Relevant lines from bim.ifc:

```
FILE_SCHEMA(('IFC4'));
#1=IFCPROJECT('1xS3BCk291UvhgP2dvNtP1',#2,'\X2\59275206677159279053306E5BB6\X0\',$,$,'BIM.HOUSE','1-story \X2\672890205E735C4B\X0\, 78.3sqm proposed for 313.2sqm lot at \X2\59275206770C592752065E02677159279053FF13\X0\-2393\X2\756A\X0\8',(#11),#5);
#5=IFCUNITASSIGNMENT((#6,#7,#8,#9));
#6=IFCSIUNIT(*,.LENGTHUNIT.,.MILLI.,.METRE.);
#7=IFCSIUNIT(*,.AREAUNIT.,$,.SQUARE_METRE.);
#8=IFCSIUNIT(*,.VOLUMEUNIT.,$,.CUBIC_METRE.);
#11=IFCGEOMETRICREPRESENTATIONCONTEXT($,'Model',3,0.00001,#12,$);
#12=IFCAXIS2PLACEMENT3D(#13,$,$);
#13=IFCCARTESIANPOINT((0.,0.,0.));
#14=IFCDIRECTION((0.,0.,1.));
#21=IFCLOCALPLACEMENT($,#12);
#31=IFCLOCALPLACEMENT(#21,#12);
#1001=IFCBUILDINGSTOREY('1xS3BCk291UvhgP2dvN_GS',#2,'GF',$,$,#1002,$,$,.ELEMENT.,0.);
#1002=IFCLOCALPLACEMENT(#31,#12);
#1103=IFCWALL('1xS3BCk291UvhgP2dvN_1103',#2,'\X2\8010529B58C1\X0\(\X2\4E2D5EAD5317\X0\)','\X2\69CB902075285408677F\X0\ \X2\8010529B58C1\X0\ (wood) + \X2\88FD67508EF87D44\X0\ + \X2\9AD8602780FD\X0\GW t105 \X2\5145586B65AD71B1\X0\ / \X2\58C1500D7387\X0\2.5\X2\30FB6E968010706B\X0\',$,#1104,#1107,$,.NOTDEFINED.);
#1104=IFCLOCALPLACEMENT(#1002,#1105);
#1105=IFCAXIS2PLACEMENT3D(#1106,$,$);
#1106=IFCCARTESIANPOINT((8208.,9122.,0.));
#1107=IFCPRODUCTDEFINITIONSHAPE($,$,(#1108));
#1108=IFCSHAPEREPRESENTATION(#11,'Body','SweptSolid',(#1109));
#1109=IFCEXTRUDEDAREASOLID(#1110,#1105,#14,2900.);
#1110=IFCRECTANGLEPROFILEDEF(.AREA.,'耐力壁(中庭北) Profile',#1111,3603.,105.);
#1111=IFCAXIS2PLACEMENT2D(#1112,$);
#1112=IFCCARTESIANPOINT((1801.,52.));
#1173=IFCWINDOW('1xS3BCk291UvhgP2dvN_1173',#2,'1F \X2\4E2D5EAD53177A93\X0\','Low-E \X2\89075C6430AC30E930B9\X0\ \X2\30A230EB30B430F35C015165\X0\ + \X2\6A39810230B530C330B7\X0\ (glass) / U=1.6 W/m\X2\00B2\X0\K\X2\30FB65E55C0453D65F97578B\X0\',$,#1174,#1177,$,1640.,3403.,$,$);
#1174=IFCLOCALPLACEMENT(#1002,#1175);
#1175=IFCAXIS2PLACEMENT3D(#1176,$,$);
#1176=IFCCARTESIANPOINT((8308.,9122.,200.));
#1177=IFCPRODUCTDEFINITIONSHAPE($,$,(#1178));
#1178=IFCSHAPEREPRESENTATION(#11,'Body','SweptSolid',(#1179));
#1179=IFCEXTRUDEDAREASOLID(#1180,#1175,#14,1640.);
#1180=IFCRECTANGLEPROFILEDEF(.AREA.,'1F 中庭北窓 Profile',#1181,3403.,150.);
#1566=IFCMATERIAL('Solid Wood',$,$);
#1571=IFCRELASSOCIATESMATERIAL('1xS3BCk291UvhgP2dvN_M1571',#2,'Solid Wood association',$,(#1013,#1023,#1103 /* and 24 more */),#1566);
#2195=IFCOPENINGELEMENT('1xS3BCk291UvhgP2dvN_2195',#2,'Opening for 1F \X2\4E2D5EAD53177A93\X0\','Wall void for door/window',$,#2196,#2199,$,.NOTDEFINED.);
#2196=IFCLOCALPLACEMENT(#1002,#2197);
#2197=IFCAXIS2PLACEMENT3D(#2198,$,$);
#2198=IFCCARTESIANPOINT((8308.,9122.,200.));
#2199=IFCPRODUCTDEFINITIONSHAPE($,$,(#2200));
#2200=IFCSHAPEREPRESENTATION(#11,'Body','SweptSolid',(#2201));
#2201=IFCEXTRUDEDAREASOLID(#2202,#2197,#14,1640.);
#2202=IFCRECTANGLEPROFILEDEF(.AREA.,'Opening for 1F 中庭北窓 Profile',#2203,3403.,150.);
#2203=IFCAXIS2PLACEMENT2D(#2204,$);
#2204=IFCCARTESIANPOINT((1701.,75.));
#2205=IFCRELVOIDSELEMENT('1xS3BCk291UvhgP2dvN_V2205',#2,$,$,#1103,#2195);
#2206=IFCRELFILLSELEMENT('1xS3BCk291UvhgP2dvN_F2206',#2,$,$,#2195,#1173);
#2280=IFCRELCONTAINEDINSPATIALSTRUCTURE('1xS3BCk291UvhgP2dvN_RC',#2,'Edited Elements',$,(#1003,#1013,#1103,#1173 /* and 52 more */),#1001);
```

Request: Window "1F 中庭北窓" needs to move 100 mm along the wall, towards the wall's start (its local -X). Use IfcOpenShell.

```python
import ifcopenshell
import ifcopenshell.api.geometry
import ifcopenshell.util.placement
import ifcopenshell.util.unit

model = ifcopenshell.open("bim.ifc")
unit_scale = ifcopenshell.util.unit.calculate_unit_scale(model)

window = model.by_id(1173)
opening = window.FillsVoids[0].RelatingOpeningElement
wall = opening.VoidsElements[0].RelatingBuildingElement

wall_matrix = ifcopenshell.util.placement.get_local_placement(wall.ObjectPlacement)
shift = wall_matrix[:3, 0] * -0.1 / unit_scale
before = ifcopenshell.util.placement.get_local_placement(window.ObjectPlacement)[:3, 3].copy()

# The window is not placed relative to its opening, so move both.
for product in (opening, window):
    matrix = ifcopenshell.util.placement.get_local_placement(product.ObjectPlacement)
    matrix[:3, 3] += shift
    ifcopenshell.api.geometry.edit_object_placement(model, product=product, matrix=matrix, is_si=False)

after = ifcopenshell.util.placement.get_local_placement(window.ObjectPlacement)[:3, 3]
print("window moved by", (after - before).round(3) + 0.0)

model.write("bim_rev.ifc")
```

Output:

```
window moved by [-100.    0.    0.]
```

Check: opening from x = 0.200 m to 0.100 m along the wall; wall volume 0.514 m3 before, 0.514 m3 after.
